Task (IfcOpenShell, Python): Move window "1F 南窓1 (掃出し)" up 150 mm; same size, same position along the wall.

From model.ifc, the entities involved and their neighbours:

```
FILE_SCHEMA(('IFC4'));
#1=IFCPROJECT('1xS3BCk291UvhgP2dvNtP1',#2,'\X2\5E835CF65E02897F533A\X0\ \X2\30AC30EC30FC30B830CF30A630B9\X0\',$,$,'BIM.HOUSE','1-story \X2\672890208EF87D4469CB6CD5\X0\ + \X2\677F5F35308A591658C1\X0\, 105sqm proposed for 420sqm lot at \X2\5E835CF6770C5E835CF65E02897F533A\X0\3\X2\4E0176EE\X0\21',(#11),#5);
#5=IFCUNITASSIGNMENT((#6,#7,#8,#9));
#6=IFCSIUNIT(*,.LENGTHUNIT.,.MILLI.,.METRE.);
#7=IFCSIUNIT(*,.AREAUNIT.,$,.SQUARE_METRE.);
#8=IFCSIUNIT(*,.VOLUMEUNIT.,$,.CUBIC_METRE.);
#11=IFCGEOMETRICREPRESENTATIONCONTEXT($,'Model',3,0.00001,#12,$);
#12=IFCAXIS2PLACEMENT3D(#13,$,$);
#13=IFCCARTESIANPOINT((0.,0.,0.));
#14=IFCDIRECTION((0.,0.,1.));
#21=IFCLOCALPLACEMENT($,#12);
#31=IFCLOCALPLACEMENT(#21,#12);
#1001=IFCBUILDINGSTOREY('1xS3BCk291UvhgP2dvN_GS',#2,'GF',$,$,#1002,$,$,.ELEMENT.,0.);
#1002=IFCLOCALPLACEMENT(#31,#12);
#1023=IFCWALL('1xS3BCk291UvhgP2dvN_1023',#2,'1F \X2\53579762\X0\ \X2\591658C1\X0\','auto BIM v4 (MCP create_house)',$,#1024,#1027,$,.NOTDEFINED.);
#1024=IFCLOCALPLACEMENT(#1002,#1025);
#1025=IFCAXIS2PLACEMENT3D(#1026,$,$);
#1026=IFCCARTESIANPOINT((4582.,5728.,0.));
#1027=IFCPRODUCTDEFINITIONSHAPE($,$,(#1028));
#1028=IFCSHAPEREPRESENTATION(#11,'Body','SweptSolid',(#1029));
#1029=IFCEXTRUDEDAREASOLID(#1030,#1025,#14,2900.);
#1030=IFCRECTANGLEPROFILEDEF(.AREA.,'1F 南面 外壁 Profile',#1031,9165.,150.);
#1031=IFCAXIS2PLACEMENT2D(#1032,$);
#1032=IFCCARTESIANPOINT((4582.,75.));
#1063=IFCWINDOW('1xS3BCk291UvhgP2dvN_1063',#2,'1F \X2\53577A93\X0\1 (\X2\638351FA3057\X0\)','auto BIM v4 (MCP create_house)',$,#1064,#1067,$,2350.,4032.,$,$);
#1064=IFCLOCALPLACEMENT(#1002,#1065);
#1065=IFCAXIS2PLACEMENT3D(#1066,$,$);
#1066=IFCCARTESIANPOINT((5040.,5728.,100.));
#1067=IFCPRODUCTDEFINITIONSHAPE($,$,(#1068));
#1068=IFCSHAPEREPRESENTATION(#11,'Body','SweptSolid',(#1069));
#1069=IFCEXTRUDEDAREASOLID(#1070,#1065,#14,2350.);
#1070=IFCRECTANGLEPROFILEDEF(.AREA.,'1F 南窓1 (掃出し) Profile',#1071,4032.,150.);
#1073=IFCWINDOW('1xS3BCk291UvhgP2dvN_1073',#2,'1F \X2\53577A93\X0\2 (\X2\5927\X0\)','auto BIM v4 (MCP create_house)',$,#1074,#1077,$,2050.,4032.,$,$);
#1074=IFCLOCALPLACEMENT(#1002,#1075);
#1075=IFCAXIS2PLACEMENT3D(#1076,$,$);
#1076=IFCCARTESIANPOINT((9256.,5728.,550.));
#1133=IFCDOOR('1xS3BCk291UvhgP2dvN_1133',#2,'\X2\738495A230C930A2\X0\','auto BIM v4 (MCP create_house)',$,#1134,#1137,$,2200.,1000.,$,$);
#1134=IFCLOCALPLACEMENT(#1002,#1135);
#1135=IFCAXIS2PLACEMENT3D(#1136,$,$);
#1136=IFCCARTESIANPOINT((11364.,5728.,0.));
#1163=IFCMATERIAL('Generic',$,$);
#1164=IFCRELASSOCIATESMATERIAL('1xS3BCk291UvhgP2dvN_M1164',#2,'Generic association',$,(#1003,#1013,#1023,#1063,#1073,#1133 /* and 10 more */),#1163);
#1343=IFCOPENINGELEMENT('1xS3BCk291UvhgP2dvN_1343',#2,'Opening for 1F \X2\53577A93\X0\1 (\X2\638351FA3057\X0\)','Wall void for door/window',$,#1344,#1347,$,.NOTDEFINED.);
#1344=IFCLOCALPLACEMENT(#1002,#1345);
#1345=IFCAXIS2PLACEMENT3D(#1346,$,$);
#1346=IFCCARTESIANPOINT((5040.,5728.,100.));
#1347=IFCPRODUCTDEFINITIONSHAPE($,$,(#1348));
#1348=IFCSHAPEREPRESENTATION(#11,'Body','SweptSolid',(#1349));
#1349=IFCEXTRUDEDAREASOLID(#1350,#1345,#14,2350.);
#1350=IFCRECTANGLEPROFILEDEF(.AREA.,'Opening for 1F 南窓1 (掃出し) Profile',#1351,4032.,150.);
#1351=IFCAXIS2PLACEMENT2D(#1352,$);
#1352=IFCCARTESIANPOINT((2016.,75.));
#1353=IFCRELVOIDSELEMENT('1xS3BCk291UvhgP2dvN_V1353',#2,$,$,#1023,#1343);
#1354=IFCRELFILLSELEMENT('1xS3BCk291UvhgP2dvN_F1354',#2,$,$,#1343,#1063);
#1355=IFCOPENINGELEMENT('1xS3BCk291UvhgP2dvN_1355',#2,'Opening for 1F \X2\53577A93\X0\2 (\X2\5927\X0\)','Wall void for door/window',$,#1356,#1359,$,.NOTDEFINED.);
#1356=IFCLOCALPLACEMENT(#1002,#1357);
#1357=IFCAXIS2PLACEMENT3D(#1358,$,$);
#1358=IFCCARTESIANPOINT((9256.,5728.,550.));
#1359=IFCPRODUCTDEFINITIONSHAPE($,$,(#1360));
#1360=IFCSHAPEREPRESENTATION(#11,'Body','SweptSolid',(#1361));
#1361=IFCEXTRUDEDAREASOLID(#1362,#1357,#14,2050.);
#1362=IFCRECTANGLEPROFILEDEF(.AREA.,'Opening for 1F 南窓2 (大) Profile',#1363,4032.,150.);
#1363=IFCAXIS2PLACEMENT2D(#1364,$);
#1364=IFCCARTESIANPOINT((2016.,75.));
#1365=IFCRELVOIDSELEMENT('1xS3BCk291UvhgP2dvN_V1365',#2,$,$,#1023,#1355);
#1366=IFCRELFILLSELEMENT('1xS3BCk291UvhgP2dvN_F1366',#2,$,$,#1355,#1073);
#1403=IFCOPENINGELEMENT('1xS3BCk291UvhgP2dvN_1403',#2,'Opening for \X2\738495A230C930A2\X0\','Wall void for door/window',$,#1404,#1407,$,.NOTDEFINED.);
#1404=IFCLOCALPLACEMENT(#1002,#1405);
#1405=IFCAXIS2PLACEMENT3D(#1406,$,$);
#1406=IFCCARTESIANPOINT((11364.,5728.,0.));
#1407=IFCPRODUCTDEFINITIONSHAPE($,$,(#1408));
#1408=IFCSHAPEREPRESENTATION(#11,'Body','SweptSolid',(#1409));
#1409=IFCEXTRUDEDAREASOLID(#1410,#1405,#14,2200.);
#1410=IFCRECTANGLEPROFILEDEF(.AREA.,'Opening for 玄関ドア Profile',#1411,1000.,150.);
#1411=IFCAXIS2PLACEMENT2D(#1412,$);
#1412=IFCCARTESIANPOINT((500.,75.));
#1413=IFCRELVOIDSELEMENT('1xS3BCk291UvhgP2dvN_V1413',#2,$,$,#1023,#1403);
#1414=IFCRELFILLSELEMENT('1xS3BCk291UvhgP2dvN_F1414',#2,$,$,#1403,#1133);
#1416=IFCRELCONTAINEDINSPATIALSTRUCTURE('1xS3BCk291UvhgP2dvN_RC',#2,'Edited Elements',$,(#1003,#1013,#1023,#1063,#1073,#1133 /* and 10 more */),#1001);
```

```python
import numpy as np
import ifcopenshell
import ifcopenshell.api.geometry
import ifcopenshell.util.placement
import ifcopenshell.util.unit

model = ifcopenshell.open("model.ifc")
unit_scale = ifcopenshell.util.unit.calculate_unit_scale(model)

window = model.by_guid("1xS3BCk291UvhgP2dvN_1063")
opening = window.FillsVoids[0].RelatingOpeningElement
dz = 0.15 / unit_scale

shift = np.array([0.0, 0.0, dz])
# The window is not placed relative to its opening, so move both.
for product in (opening, window):
    matrix = ifcopenshell.util.placement.get_local_placement(product.ObjectPlacement)
    matrix[:3, 3] += shift
    ifcopenshell.api.geometry.edit_object_placement(model, product=product, matrix=matrix, is_si=False)

print(f"moved by {dz * unit_scale:+.3f} m")

model.write("model_updated.ifc")
```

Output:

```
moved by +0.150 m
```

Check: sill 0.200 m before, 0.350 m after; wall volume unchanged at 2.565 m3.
